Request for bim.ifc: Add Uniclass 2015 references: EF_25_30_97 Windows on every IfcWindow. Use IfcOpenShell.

First a look at what the model holds.

```python
import ifcopenshell

model = ifcopenshell.open("bim.ifc")
print(model.schema)
print("classifications:", [c.Name for c in model.by_type("IfcClassification")])
for ifc_class in ("IfcDoor", "IfcRoof", "IfcStair", "IfcWall", "IfcWindow"):
    print(ifc_class, len(model.by_type(ifc_class)))
```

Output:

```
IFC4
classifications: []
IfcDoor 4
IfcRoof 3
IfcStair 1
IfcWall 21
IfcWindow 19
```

```python
import ifcopenshell
import ifcopenshell.api.classification

model = ifcopenshell.open("bim.ifc")

system = ifcopenshell.api.classification.add_classification(model, classification="Uniclass 2015")

codes = {
    "IfcWindow": ("EF_25_30_97", "Windows"),
}
for ifc_class, (code, name) in codes.items():
    products = model.by_type(ifc_class)
    ifcopenshell.api.classification.add_reference(
        model, products=products, classification=system, identification=code, name=name
    )
    print(code, len(products))

model.write("bim_edited.ifc")
```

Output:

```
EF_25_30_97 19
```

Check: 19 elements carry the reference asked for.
